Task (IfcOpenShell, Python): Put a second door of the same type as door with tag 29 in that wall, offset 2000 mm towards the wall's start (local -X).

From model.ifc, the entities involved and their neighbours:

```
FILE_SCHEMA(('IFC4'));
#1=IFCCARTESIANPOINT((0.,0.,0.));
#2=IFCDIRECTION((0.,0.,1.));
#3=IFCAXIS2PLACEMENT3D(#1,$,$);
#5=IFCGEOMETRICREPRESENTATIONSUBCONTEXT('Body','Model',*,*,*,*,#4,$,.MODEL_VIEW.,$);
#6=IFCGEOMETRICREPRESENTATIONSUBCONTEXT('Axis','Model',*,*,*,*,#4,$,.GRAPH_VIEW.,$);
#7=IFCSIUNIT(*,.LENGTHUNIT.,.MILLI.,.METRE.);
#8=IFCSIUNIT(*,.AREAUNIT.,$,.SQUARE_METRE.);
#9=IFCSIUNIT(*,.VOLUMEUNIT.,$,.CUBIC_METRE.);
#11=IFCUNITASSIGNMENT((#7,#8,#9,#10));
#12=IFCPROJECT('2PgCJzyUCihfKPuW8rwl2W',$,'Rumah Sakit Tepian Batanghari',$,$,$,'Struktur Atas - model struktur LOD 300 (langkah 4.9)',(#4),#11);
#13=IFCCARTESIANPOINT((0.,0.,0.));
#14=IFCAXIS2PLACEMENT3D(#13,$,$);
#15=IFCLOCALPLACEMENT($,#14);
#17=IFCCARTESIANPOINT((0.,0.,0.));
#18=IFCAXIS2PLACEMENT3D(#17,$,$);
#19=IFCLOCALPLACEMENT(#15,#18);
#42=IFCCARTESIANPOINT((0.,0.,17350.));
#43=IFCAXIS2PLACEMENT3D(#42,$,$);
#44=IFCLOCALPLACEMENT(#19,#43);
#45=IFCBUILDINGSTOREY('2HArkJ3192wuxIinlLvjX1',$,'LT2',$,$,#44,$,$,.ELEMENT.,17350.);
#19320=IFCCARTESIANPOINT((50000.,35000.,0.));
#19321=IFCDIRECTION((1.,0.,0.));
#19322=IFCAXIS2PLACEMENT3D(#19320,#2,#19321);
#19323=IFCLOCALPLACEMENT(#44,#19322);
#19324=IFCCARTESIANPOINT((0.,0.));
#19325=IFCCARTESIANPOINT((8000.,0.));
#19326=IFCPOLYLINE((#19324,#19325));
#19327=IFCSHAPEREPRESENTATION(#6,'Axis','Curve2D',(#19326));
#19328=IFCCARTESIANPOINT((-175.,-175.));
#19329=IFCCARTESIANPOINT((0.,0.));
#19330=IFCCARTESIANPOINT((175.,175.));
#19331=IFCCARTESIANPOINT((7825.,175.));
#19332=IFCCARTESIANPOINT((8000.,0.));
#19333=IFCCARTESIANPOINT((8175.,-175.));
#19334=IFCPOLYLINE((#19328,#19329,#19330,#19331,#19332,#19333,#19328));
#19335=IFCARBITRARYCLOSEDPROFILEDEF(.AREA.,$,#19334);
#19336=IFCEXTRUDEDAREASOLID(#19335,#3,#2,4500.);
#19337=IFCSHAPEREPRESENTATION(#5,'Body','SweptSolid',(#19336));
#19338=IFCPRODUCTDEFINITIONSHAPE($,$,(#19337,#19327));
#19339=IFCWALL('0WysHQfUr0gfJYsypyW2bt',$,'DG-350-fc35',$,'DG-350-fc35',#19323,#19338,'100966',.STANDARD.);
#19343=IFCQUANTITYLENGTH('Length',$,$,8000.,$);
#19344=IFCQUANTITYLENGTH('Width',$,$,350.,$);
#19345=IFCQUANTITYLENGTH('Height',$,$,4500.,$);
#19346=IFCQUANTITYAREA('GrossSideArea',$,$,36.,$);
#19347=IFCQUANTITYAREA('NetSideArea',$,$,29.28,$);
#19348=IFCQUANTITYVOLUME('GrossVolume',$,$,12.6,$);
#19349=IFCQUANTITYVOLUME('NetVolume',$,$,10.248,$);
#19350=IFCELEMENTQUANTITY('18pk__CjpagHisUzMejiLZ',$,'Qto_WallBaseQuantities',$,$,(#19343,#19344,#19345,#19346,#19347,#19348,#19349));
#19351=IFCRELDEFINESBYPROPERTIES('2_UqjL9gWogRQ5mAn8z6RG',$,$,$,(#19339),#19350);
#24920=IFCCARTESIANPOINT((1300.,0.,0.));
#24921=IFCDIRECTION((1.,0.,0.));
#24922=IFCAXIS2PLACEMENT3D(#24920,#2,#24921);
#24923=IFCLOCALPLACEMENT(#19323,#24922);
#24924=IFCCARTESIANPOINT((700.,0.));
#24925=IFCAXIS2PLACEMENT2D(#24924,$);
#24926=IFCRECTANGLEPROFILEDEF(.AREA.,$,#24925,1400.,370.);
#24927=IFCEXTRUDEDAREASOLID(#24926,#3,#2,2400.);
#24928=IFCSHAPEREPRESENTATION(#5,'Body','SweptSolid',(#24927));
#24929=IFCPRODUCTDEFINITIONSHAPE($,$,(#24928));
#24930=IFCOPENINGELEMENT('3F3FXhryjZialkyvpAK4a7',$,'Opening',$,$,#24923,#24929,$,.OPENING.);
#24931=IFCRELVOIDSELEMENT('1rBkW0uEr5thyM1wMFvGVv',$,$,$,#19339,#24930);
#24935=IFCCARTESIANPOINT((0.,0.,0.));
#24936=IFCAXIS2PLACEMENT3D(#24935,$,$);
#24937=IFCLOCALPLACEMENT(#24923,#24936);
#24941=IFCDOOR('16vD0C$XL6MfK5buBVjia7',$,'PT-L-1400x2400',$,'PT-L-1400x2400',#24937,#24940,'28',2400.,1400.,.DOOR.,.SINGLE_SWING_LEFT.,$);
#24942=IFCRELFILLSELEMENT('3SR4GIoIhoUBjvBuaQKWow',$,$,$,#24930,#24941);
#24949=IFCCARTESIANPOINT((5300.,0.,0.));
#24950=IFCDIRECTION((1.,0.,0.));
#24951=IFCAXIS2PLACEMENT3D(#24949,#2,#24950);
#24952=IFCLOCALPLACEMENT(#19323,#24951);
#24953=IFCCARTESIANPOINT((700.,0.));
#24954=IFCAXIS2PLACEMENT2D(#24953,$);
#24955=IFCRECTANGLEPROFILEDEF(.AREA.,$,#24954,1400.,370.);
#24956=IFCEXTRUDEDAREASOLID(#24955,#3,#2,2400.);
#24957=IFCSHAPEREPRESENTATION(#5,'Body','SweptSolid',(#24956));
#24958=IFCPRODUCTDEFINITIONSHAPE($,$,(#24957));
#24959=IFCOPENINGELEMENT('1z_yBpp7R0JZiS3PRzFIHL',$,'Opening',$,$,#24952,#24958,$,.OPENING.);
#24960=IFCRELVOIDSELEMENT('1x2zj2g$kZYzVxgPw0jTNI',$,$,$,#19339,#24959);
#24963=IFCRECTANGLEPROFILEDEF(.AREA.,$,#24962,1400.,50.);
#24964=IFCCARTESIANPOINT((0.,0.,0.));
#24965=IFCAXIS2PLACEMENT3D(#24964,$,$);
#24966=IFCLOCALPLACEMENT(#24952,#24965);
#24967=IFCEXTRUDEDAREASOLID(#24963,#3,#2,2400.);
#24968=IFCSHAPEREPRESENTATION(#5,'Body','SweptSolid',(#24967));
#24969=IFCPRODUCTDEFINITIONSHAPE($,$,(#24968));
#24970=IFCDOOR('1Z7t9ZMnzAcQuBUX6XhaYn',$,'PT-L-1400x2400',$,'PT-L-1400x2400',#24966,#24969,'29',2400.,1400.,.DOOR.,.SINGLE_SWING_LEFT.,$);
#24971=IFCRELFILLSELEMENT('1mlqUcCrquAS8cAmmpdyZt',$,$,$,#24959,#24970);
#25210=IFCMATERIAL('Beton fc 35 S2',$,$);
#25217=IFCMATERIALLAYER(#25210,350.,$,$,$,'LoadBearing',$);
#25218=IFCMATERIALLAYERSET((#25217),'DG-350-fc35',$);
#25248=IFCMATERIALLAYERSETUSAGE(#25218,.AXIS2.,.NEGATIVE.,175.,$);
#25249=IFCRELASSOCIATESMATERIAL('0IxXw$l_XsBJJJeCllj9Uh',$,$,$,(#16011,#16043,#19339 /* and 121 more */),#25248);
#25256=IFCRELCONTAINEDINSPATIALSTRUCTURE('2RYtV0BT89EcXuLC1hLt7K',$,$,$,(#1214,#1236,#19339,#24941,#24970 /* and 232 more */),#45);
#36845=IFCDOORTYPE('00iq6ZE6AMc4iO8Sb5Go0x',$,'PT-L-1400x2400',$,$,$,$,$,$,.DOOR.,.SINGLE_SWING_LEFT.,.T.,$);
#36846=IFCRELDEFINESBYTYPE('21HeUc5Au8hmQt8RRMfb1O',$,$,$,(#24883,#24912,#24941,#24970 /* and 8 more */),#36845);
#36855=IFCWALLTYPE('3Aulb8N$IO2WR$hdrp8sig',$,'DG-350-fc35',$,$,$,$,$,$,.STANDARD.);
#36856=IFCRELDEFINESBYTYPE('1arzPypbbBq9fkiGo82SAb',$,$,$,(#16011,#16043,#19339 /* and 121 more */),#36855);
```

```python
import ifcopenshell
import ifcopenshell.api.feature
import ifcopenshell.api.geometry
import ifcopenshell.api.pset
import ifcopenshell.api.root
import ifcopenshell.geom
import ifcopenshell.util.element
import ifcopenshell.util.placement
import ifcopenshell.util.shape
import ifcopenshell.util.unit

model = ifcopenshell.open("model.ifc")
area_scale = ifcopenshell.util.unit.calculate_unit_scale(model, "AREAUNIT")
volume_scale = ifcopenshell.util.unit.calculate_unit_scale(model, "VOLUMEUNIT")
settings = ifcopenshell.geom.settings()


def volume(element):
    """Net volume in cubic metres, openings subtracted."""
    shape = ifcopenshell.geom.create_shape(settings, element)
    return ifcopenshell.util.shape.get_volume(shape.geometry)


door = model.by_guid("1Z7t9ZMnzAcQuBUX6XhaYn")
opening = door.FillsVoids[0].RelatingOpeningElement
wall = opening.VoidsElements[0].RelatingBuildingElement
before = volume(wall)
shift = ifcopenshell.util.placement.get_local_placement(wall.ObjectPlacement)[:3, 0] * -2000.0

# copy_class copies the void relationship, type, container and properties, but no geometry.
new_opening = ifcopenshell.api.root.copy_class(model, product=opening)
new_opening.Representation = ifcopenshell.util.element.copy_deep(
    model, opening.Representation, exclude=["IfcGeometricRepresentationContext", "IfcRepresentationMap"]
)
new_door = ifcopenshell.api.root.copy_class(model, product=door)
new_door.Representation = ifcopenshell.util.element.copy_deep(
    model, door.Representation, exclude=["IfcGeometricRepresentationContext", "IfcRepresentationMap"]
)
new_door.Tag = None
ifcopenshell.api.feature.add_filling(model, opening=new_opening, element=new_door)

for old, new in ((opening, new_opening), (door, new_door)):
    matrix = ifcopenshell.util.placement.get_local_placement(old.ObjectPlacement)
    matrix[:3, 3] += shift
    ifcopenshell.api.geometry.edit_object_placement(model, product=new, matrix=matrix, is_si=False)

after = volume(wall)
thickness = 0.35  # wall thickness in metres

# Update the wall's stored quantities.
qto = model.by_id(ifcopenshell.util.element.get_pset(wall, "Qto_WallBaseQuantities", should_inherit=False)["id"])
ifcopenshell.api.pset.edit_qto(model, qto=qto, properties={
    "NetSideArea": after / thickness / area_scale,
    "NetVolume": after / volume_scale,
})

print(f"wall volume {before:.3f} -> {after:.3f} m3")

model.write("model_edited.ifc")
```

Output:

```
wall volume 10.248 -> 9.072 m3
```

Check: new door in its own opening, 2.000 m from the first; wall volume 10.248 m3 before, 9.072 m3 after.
